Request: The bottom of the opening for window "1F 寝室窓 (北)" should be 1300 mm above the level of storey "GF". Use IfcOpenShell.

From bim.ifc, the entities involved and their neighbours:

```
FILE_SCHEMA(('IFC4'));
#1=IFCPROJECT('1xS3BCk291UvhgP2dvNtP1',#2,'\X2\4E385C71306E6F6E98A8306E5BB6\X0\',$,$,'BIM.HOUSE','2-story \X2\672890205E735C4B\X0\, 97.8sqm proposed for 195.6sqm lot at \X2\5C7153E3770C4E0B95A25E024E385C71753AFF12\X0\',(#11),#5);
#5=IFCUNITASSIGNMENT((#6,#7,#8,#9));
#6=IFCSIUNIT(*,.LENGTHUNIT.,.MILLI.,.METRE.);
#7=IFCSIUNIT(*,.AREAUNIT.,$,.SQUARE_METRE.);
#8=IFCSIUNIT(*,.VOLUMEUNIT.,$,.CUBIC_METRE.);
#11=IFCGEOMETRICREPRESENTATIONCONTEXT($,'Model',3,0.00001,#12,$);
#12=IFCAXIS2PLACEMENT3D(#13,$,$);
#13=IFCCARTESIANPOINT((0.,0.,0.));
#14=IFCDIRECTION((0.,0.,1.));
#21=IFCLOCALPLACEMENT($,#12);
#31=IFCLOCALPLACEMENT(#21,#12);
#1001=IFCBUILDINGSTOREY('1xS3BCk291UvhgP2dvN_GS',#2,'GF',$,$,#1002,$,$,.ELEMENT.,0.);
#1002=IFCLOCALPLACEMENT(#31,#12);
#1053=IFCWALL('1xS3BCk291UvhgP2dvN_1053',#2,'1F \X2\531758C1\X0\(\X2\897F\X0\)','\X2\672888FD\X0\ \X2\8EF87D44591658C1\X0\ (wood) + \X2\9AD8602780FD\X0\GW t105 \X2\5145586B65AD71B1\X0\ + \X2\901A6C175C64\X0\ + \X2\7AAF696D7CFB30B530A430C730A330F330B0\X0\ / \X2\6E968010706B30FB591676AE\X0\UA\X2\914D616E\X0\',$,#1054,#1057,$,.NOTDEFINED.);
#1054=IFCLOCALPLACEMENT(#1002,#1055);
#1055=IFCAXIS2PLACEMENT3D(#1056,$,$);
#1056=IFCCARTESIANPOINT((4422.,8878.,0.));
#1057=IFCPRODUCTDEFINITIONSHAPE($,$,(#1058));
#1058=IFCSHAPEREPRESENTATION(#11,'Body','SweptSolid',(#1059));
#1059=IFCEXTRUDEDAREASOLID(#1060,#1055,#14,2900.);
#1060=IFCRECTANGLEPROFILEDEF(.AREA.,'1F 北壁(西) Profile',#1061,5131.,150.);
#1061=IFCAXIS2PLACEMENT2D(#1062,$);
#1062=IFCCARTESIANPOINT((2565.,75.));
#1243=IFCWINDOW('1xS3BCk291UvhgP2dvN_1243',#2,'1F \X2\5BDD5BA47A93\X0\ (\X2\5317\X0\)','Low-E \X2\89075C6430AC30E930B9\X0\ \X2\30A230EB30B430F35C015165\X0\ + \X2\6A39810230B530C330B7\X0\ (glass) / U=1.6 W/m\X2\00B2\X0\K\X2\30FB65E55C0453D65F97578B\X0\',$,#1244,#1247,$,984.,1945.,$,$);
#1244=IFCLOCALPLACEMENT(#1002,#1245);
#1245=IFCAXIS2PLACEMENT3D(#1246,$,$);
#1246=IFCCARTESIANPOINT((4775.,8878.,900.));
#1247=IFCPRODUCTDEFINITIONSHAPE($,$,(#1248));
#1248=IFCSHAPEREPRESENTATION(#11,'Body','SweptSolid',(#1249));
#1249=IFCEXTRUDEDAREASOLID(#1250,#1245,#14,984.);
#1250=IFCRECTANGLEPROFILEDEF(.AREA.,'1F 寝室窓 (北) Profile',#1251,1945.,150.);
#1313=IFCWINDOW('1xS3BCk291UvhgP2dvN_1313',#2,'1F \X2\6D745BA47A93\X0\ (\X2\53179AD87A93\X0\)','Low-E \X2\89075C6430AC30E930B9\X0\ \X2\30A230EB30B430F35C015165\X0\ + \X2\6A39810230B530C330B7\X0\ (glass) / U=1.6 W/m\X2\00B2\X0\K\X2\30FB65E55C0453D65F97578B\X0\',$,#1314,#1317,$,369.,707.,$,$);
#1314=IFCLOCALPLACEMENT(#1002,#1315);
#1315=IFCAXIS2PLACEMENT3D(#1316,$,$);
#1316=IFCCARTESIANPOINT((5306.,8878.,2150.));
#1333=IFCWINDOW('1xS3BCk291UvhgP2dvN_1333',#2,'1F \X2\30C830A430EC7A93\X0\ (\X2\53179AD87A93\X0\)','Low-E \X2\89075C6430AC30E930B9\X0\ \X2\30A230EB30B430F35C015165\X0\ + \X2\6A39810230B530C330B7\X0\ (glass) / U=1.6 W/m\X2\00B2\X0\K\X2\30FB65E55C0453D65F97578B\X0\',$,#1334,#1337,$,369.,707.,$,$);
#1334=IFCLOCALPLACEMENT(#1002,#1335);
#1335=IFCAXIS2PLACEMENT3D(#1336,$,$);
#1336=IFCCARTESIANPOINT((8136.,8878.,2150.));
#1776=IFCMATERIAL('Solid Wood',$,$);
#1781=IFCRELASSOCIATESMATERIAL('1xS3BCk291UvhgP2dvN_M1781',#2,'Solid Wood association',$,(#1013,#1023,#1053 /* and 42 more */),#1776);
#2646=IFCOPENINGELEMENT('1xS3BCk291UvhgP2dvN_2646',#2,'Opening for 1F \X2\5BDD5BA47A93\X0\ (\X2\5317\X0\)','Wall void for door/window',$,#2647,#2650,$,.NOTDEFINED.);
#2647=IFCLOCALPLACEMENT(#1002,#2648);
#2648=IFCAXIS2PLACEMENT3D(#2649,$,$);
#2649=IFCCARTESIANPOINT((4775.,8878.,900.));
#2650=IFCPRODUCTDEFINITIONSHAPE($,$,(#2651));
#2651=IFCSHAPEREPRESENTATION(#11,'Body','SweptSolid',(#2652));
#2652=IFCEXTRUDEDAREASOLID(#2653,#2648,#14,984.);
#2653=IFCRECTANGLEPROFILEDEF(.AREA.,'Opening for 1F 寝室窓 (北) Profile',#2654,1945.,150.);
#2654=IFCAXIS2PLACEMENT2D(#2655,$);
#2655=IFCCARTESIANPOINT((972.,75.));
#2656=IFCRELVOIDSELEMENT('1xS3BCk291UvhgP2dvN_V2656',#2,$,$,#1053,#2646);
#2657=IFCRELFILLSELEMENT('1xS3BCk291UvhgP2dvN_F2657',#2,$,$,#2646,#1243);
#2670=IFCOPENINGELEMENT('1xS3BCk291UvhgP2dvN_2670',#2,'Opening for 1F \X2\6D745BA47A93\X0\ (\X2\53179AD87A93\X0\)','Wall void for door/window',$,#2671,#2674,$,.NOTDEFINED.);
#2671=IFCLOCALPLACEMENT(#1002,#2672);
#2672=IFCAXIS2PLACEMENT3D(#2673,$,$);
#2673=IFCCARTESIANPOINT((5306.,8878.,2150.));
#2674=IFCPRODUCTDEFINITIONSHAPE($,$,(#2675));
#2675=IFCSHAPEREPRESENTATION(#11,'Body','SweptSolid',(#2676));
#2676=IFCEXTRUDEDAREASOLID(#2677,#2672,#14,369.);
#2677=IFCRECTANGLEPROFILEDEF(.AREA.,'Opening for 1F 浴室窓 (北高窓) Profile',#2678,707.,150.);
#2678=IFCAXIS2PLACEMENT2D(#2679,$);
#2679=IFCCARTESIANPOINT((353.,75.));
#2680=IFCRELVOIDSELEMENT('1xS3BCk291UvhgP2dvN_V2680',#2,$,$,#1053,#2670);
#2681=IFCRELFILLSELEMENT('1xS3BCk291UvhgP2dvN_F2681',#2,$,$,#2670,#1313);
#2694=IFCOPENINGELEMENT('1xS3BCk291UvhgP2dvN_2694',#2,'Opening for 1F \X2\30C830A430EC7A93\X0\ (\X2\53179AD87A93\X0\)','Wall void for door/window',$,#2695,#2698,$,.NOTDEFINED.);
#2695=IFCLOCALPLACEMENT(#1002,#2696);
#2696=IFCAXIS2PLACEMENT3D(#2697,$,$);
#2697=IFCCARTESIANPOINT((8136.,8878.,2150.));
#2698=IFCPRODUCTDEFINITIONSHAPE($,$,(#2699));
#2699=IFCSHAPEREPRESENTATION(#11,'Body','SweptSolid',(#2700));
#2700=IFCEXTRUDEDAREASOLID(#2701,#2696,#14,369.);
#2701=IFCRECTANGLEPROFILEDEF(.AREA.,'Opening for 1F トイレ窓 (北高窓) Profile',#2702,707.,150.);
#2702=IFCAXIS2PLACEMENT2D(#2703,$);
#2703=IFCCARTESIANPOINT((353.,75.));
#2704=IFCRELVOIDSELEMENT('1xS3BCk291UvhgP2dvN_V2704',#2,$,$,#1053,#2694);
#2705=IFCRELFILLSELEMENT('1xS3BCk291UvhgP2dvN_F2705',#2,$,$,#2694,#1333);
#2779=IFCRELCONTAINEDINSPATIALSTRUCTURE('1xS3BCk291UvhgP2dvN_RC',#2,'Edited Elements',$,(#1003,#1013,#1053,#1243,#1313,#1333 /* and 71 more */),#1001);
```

```python
import numpy as np
import ifcopenshell
import ifcopenshell.api.geometry
import ifcopenshell.geom
import ifcopenshell.util.element
import ifcopenshell.util.placement
import ifcopenshell.util.shape
import ifcopenshell.util.unit

model = ifcopenshell.open("bim.ifc")
unit_scale = ifcopenshell.util.unit.calculate_unit_scale(model)

window = model.by_id(1243)
opening = window.FillsVoids[0].RelatingOpeningElement
storey = ifcopenshell.util.element.get_container(window, ifc_class="IfcBuildingStorey")
level = ifcopenshell.util.placement.get_local_placement(storey.ObjectPlacement)[2, 3]

# The opening's origin need not be at the sill, so measure its lowest point.
shape = ifcopenshell.geom.create_shape(ifcopenshell.geom.settings(), opening)
bottom = ifcopenshell.util.shape.get_shape_bottom_elevation(shape, shape.geometry) / unit_scale
dz = level + 1.3 / unit_scale - bottom

shift = np.array([0.0, 0.0, dz])
# The window is not placed relative to its opening, so move both.
for product in (opening, window):
    matrix = ifcopenshell.util.placement.get_local_placement(product.ObjectPlacement)
    matrix[:3, 3] += shift
    ifcopenshell.api.geometry.edit_object_placement(model, product=product, matrix=matrix, is_si=False)

print(f"moved by {dz * unit_scale:+.3f} m")

model.write("bim_edited.ifc")
```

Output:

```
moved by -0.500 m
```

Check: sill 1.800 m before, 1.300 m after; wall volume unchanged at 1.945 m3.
